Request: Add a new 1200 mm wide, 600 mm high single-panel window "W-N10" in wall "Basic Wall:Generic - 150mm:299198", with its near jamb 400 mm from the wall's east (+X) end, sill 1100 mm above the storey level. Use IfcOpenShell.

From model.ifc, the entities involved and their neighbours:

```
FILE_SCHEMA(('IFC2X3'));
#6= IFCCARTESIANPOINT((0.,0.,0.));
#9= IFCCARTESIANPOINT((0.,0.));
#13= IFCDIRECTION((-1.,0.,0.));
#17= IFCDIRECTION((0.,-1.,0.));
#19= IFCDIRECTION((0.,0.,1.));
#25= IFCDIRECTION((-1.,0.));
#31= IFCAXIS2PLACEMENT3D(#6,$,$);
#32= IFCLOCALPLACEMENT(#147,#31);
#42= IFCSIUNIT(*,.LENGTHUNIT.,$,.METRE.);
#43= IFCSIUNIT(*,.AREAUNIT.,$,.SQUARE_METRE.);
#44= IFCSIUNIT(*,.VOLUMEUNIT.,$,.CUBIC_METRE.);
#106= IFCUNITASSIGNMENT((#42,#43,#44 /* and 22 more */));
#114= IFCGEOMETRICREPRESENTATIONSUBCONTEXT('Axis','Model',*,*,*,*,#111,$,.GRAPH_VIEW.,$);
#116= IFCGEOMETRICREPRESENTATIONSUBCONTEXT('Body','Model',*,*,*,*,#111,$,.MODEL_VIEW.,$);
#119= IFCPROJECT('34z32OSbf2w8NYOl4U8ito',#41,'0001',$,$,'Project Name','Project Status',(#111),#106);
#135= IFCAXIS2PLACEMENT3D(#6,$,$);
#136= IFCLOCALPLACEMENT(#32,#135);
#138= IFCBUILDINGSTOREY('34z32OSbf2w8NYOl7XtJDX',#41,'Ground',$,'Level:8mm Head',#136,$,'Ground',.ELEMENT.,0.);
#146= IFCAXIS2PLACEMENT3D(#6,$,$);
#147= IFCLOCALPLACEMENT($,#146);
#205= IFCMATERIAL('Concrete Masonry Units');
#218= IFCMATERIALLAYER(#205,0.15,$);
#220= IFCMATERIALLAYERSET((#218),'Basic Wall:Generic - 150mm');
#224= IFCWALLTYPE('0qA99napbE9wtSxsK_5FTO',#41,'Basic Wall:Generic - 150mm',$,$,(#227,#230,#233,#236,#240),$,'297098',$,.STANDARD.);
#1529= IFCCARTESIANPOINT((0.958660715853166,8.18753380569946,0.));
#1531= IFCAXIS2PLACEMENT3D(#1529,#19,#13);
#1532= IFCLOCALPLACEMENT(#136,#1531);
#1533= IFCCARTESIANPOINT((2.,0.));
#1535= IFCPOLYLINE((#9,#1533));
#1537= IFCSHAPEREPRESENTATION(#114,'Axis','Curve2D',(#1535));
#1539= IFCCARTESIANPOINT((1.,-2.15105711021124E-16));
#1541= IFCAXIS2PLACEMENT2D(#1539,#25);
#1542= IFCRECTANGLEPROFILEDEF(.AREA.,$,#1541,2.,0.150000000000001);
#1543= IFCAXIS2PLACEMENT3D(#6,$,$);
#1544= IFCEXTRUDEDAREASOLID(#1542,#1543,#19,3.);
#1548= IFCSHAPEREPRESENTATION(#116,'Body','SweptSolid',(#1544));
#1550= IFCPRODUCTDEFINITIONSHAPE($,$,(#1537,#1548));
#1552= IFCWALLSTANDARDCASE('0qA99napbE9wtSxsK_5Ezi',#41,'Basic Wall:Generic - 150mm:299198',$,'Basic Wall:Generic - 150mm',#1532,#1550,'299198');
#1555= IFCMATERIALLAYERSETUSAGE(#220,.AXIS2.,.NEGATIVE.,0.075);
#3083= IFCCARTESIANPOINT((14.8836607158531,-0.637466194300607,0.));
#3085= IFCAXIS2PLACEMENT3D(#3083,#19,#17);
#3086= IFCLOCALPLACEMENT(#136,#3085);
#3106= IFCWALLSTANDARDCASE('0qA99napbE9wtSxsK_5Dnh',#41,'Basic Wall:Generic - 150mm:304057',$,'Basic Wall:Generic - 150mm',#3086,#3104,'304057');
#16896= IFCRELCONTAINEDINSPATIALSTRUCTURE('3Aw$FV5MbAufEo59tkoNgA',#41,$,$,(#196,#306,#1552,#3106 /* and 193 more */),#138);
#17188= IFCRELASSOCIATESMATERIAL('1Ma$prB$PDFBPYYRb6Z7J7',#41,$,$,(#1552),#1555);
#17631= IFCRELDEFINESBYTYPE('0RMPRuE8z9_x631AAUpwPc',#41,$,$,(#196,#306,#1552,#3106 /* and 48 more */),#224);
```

```python
import numpy as np
import ifcopenshell
import ifcopenshell.api.feature
import ifcopenshell.api.geometry
import ifcopenshell.api.root
import ifcopenshell.api.spatial
import ifcopenshell.api.type
import ifcopenshell.geom
import ifcopenshell.util.element
import ifcopenshell.util.placement
import ifcopenshell.util.representation
import ifcopenshell.util.shape
import ifcopenshell.util.unit

model = ifcopenshell.open("model.ifc")
unit_scale = ifcopenshell.util.unit.calculate_unit_scale(model)
settings = ifcopenshell.geom.settings()


def volume(element):
    """Net volume in cubic metres, openings subtracted."""
    shape = ifcopenshell.geom.create_shape(settings, element)
    return ifcopenshell.util.shape.get_volume(shape.geometry)


wall = model.by_guid("0qA99napbE9wtSxsK_5Ezi")
storey = ifcopenshell.util.element.get_container(wall, ifc_class="IfcBuildingStorey")
context = ifcopenshell.util.representation.get_context(model, "Model", "Body", "MODEL_VIEW")
before = volume(wall)

width, height, from_end, sill = 1.2, 0.6, 0.4, 1.1  # metres

# The wall runs along its own X axis, and the end named is its -X end.
wall_shape = ifcopenshell.geom.create_shape(settings, wall)
x, y, z = ifcopenshell.util.shape.get_vertices(wall_shape.geometry).T
start = x.min() + from_end
face, thickness = float(y.min()), float(y.max() - y.min())
wall_matrix = ifcopenshell.util.placement.get_local_placement(wall.ObjectPlacement)
level = ifcopenshell.util.placement.get_local_placement(storey.ObjectPlacement)[2, 3]


def in_wall(x, y):
    """Placement at x, y metres in the wall's axes, at sill height."""
    matrix = wall_matrix.copy()
    matrix[:, 3] = wall_matrix @ np.array([x / unit_scale, y / unit_scale, 0.0, 1.0])
    matrix[2, 3] = level + sill / unit_scale
    return matrix


# Opening: a box that overshoots both wall faces by 50 mm.
opening = ifcopenshell.api.root.create_entity(model, ifc_class="IfcOpeningElement")
box = ifcopenshell.api.geometry.add_wall_representation(
    model, context=context, length=width, height=height, thickness=thickness + 0.1
)
ifcopenshell.api.geometry.assign_representation(model, product=opening, representation=box)
ifcopenshell.api.geometry.edit_object_placement(model, product=opening, matrix=in_wall(start, face - 0.05), is_si=False)
ifcopenshell.api.feature.add_feature(model, feature=opening, element=wall)

window = ifcopenshell.api.root.create_entity(model, ifc_class="IfcWindow", name="W-N10")
window.OverallWidth, window.OverallHeight = width / unit_scale, height / unit_scale
body = ifcopenshell.api.geometry.add_window_representation(
    model,
    context=context,
    overall_width=window.OverallWidth,
    overall_height=window.OverallHeight,
    partition_type="SINGLE_PANEL",
)
ifcopenshell.api.geometry.assign_representation(model, product=window, representation=body)
ifcopenshell.api.spatial.assign_container(model, products=[window], relating_structure=storey)
fills = ifcopenshell.api.feature.add_filling(model, opening=opening, element=window)
fills.OwnerHistory = window.OwnerHistory  # required in IFC2X3

# IFC2X3 keeps the operation on the window style.
style = ifcopenshell.api.root.create_entity(model, ifc_class="IfcWindowStyle", name="W-N10")
style.OperationType, style.ConstructionType = "SINGLE_PANEL", "NOTDEFINED"
style.ParameterTakesPrecedence = style.Sizeable = False
ifcopenshell.api.type.assign_type(model, related_objects=[window], relating_type=style)

# Centre the window in the wall's thickness.
ifcopenshell.api.geometry.edit_object_placement(model, product=window, matrix=in_wall(start, face), is_si=False)
window_shape = ifcopenshell.geom.create_shape(settings, window)
depth = ifcopenshell.util.shape.get_vertices(window_shape.geometry)[:, 1]
offset = face + thickness / 2 - (depth.min() + depth.max()) / 2
ifcopenshell.api.geometry.edit_object_placement(model, product=window, matrix=in_wall(start, offset), is_si=False)

after = volume(wall)

print(f"wall volume {before:.3f} -> {after:.3f} m3")

model.write("model-out.ifc")
```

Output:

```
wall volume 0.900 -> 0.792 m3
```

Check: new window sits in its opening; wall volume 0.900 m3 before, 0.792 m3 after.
